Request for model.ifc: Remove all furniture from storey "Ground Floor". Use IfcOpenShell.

First a look at what the model holds.

```python
import ifcopenshell
import ifcopenshell.util.element

model = ifcopenshell.open("model.ifc")
print(model.schema)
storey = next(s for s in model.by_type("IfcBuildingStorey") if s.Name == "Ground Floor")
furniture = [e for e in ifcopenshell.util.element.get_decomposition(storey) if e.is_a("IfcFurnishingElement")]
seen = {}
for e in furniture:
    element_type = ifcopenshell.util.element.get_type(e)
    name = element_type.Name if element_type not in (None, e) else None
    seen[name] = seen.get(name, 0) + 1
for name, count in sorted(seen.items(), key=str):
    print(count, "x", name)
```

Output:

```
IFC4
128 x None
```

```python
import ifcopenshell
import ifcopenshell.api.root
import ifcopenshell.util.element

model = ifcopenshell.open("model.ifc")

storey = next(s for s in model.by_type("IfcBuildingStorey") if s.Name == "Ground Floor")
furniture = [e for e in ifcopenshell.util.element.get_decomposition(storey) if e.is_a("IfcFurnishingElement")]

for e in furniture:
    ifcopenshell.api.root.remove_product(model, product=e)
print(len(furniture), "removed")

model.write("model_rev.ifc")
```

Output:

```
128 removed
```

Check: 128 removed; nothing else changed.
